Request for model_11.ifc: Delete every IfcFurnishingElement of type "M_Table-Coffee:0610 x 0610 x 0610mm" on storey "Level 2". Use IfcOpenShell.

First a look at what the model holds.

```python
import ifcopenshell
import ifcopenshell.util.element

model = ifcopenshell.open("model_11.ifc")
print(model.schema)
storey = next(s for s in model.by_type("IfcBuildingStorey") if s.Name == "Level 2")
furniture = [e for e in ifcopenshell.util.element.get_decomposition(storey) if e.is_a("IfcFurnishingElement")]
seen = {}
for e in furniture:
    element_type = ifcopenshell.util.element.get_type(e)
    name = element_type.Name if element_type not in (None, e) else None
    seen[name] = seen.get(name, 0) + 1
for name, count in sorted(seen.items(), key=str):
    print(count, "x", name)
```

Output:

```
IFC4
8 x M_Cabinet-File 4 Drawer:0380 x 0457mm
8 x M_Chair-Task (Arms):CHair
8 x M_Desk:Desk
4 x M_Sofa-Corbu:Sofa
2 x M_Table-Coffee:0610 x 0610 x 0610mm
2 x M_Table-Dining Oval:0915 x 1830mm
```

```python
import ifcopenshell
import ifcopenshell.api.root
import ifcopenshell.util.element

model = ifcopenshell.open("model_11.ifc")

storey = next(s for s in model.by_type("IfcBuildingStorey") if s.Name == "Level 2")
furniture = [e for e in ifcopenshell.util.element.get_decomposition(storey) if e.is_a("IfcFurnishingElement")]
targets = [e for e in furniture if (t := ifcopenshell.util.element.get_type(e)) not in (None, e) and t.Name == "M_Table-Coffee:0610 x 0610 x 0610mm"]

for e in targets:
    ifcopenshell.api.root.remove_product(model, product=e)
print(len(targets), "removed")

model.write("model_11-out.ifc")
```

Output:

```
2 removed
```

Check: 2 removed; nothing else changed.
